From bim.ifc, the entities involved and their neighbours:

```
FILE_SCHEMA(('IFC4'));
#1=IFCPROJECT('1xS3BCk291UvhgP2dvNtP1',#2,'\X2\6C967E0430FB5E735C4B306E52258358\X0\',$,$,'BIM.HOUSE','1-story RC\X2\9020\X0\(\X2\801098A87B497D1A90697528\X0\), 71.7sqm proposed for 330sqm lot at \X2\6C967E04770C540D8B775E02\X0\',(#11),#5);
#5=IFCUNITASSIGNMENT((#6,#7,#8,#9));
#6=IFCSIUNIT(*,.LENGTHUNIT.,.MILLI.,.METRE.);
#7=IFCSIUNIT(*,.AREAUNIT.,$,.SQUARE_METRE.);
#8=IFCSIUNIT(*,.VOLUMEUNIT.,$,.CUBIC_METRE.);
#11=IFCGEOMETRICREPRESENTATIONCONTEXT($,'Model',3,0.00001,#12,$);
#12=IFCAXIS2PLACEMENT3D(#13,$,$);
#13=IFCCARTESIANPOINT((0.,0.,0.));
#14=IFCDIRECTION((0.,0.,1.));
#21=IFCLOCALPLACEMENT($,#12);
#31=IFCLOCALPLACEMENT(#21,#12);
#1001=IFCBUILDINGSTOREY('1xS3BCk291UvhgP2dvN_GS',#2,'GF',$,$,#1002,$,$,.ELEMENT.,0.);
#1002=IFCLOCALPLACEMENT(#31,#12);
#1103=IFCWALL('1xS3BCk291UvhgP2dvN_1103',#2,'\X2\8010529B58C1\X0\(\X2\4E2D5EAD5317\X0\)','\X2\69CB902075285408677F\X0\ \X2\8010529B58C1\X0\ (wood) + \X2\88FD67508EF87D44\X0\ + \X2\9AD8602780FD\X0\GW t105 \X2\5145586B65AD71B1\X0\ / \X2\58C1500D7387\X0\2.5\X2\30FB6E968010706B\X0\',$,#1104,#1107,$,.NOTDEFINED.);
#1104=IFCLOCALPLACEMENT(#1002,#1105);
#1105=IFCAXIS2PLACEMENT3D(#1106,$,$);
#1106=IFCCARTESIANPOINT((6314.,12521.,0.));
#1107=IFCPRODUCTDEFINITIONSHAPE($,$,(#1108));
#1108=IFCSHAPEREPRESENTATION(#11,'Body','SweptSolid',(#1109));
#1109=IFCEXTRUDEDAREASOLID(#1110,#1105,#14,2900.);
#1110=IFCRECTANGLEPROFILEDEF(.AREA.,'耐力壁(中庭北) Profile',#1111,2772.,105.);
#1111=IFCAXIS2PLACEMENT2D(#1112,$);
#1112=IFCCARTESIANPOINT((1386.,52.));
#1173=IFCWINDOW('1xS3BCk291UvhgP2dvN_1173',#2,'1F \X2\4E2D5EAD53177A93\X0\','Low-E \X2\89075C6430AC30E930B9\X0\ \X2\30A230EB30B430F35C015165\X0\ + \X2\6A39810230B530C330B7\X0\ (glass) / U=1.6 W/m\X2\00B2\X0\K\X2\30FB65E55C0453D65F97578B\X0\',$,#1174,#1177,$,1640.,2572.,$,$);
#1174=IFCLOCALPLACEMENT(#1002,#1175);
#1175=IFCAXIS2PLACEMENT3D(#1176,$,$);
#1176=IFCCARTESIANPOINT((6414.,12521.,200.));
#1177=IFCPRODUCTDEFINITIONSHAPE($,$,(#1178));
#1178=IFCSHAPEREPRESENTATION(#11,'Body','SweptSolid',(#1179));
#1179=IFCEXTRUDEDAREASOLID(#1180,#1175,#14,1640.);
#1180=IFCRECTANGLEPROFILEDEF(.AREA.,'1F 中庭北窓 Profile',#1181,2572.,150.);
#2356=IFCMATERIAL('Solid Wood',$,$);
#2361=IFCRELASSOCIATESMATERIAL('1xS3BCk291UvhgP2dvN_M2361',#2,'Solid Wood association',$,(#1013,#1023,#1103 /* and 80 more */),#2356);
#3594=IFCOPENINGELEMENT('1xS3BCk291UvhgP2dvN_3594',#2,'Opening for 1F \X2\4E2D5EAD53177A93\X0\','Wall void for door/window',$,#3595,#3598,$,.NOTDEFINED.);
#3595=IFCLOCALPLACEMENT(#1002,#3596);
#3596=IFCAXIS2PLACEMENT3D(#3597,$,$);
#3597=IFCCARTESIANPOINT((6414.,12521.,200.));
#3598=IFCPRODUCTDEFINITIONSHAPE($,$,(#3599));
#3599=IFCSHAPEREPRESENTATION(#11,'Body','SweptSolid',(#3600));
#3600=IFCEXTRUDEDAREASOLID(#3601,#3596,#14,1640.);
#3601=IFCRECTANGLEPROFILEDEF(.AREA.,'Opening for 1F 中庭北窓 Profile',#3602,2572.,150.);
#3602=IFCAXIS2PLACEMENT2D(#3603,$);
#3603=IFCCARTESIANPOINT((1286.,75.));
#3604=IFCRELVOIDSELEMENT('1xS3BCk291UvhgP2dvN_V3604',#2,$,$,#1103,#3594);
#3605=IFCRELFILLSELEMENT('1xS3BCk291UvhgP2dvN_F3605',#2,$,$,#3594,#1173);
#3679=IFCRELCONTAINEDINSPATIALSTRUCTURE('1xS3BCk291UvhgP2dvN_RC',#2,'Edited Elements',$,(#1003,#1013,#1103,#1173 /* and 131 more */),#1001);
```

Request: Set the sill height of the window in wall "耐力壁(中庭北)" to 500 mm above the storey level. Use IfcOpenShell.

```python
import numpy as np
import ifcopenshell
import ifcopenshell.api.geometry
import ifcopenshell.geom
import ifcopenshell.util.element
import ifcopenshell.util.placement
import ifcopenshell.util.shape
import ifcopenshell.util.unit

model = ifcopenshell.open("bim.ifc")
unit_scale = ifcopenshell.util.unit.calculate_unit_scale(model)

window = model.by_guid("1xS3BCk291UvhgP2dvN_1173")
opening = window.FillsVoids[0].RelatingOpeningElement
storey = ifcopenshell.util.element.get_container(window, ifc_class="IfcBuildingStorey")
level = ifcopenshell.util.placement.get_local_placement(storey.ObjectPlacement)[2, 3]

# The opening's origin need not be at the sill, so measure its lowest point.
shape = ifcopenshell.geom.create_shape(ifcopenshell.geom.settings(), opening)
bottom = ifcopenshell.util.shape.get_shape_bottom_elevation(shape, shape.geometry) / unit_scale
dz = level + 0.5 / unit_scale - bottom

shift = np.array([0.0, 0.0, dz])
# The window is not placed relative to its opening, so move both.
for product in (opening, window):
    matrix = ifcopenshell.util.placement.get_local_placement(product.ObjectPlacement)
    matrix[:3, 3] += shift
    ifcopenshell.api.geometry.edit_object_placement(model, product=product, matrix=matrix, is_si=False)

print(f"moved by {dz * unit_scale:+.3f} m")

model.write("bim_edited.ifc")
```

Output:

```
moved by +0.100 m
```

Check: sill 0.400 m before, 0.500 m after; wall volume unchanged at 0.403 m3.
